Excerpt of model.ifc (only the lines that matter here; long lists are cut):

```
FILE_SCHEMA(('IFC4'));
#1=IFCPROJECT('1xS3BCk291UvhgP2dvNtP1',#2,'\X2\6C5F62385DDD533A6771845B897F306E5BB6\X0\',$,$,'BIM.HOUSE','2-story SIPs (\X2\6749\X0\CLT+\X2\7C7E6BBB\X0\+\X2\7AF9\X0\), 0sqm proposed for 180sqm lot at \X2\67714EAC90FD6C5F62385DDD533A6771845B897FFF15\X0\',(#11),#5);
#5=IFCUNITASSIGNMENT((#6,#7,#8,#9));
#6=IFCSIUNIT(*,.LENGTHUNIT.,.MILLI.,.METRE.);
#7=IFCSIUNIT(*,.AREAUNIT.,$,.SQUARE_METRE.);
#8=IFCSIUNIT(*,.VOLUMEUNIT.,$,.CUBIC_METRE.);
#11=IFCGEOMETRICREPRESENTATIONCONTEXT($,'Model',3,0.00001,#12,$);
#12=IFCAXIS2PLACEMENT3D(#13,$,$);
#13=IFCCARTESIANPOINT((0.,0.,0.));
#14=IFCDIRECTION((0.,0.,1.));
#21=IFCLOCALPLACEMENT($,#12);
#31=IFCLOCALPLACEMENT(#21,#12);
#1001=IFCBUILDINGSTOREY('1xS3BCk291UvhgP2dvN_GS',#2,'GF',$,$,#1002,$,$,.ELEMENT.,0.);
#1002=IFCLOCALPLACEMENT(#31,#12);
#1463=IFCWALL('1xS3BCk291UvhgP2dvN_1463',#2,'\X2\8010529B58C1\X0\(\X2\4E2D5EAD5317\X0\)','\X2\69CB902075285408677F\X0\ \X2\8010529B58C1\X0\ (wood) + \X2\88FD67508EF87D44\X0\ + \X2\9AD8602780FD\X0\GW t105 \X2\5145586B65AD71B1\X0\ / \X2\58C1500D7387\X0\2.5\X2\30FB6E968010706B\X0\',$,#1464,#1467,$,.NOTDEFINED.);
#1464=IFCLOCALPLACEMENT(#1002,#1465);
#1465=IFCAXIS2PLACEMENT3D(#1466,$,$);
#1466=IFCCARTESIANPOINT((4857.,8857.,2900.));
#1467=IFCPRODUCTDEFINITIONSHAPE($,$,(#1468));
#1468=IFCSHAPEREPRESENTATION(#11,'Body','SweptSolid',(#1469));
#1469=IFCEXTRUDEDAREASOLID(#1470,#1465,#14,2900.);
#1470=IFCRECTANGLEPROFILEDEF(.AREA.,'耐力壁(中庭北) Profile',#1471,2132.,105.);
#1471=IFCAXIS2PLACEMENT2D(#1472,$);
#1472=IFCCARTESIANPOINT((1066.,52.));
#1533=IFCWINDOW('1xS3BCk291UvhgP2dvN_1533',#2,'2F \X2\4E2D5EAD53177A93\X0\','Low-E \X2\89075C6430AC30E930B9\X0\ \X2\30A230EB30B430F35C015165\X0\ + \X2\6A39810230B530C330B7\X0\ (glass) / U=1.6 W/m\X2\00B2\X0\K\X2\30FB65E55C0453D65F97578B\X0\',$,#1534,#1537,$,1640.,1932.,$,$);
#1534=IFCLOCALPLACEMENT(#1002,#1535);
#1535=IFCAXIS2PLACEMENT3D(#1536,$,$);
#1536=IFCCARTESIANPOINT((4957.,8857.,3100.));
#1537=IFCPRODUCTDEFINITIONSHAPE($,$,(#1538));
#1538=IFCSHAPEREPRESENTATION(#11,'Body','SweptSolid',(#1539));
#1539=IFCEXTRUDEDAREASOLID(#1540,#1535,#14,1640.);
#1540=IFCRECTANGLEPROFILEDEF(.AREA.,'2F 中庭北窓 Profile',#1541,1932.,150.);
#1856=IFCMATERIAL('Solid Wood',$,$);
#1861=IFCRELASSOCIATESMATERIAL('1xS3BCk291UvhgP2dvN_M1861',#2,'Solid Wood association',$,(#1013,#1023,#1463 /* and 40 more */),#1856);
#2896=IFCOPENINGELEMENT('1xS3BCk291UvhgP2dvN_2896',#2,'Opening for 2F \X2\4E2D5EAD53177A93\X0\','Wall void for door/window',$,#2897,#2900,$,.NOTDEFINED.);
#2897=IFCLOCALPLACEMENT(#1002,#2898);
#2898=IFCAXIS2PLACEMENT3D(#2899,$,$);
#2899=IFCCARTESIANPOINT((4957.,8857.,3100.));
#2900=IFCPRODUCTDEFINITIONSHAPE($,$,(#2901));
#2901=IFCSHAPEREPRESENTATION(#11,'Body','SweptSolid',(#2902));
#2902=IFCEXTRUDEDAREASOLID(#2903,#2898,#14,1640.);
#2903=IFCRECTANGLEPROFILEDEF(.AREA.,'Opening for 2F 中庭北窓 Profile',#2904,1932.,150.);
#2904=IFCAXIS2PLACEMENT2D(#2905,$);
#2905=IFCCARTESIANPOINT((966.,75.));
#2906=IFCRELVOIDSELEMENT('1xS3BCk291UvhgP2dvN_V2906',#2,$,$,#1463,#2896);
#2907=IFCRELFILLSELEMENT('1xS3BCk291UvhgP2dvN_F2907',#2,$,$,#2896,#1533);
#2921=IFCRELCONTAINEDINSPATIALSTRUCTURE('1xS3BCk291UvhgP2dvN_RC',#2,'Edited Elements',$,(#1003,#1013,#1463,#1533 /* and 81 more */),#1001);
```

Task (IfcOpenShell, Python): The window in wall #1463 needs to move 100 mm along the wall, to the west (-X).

```python
import ifcopenshell
import ifcopenshell.api.geometry
import ifcopenshell.util.placement

model = ifcopenshell.open("model.ifc")

window = model.by_guid("1xS3BCk291UvhgP2dvN_1533")
opening = window.FillsVoids[0].RelatingOpeningElement
wall = opening.VoidsElements[0].RelatingBuildingElement

wall_matrix = ifcopenshell.util.placement.get_local_placement(wall.ObjectPlacement)
shift = wall_matrix[:3, 0] * -100.0
before = ifcopenshell.util.placement.get_local_placement(window.ObjectPlacement)[:3, 3].copy()

# The window is not placed relative to its opening, so move both.
for product in (opening, window):
    matrix = ifcopenshell.util.placement.get_local_placement(product.ObjectPlacement)
    matrix[:3, 3] += shift
    ifcopenshell.api.geometry.edit_object_placement(model, product=product, matrix=matrix, is_si=False)

after = ifcopenshell.util.placement.get_local_placement(window.ObjectPlacement)[:3, 3]
print("window moved by", (after - before).round(3) + 0.0)

model.write("model_rev.ifc")
```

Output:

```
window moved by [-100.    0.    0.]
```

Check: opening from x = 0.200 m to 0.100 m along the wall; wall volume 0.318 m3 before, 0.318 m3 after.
